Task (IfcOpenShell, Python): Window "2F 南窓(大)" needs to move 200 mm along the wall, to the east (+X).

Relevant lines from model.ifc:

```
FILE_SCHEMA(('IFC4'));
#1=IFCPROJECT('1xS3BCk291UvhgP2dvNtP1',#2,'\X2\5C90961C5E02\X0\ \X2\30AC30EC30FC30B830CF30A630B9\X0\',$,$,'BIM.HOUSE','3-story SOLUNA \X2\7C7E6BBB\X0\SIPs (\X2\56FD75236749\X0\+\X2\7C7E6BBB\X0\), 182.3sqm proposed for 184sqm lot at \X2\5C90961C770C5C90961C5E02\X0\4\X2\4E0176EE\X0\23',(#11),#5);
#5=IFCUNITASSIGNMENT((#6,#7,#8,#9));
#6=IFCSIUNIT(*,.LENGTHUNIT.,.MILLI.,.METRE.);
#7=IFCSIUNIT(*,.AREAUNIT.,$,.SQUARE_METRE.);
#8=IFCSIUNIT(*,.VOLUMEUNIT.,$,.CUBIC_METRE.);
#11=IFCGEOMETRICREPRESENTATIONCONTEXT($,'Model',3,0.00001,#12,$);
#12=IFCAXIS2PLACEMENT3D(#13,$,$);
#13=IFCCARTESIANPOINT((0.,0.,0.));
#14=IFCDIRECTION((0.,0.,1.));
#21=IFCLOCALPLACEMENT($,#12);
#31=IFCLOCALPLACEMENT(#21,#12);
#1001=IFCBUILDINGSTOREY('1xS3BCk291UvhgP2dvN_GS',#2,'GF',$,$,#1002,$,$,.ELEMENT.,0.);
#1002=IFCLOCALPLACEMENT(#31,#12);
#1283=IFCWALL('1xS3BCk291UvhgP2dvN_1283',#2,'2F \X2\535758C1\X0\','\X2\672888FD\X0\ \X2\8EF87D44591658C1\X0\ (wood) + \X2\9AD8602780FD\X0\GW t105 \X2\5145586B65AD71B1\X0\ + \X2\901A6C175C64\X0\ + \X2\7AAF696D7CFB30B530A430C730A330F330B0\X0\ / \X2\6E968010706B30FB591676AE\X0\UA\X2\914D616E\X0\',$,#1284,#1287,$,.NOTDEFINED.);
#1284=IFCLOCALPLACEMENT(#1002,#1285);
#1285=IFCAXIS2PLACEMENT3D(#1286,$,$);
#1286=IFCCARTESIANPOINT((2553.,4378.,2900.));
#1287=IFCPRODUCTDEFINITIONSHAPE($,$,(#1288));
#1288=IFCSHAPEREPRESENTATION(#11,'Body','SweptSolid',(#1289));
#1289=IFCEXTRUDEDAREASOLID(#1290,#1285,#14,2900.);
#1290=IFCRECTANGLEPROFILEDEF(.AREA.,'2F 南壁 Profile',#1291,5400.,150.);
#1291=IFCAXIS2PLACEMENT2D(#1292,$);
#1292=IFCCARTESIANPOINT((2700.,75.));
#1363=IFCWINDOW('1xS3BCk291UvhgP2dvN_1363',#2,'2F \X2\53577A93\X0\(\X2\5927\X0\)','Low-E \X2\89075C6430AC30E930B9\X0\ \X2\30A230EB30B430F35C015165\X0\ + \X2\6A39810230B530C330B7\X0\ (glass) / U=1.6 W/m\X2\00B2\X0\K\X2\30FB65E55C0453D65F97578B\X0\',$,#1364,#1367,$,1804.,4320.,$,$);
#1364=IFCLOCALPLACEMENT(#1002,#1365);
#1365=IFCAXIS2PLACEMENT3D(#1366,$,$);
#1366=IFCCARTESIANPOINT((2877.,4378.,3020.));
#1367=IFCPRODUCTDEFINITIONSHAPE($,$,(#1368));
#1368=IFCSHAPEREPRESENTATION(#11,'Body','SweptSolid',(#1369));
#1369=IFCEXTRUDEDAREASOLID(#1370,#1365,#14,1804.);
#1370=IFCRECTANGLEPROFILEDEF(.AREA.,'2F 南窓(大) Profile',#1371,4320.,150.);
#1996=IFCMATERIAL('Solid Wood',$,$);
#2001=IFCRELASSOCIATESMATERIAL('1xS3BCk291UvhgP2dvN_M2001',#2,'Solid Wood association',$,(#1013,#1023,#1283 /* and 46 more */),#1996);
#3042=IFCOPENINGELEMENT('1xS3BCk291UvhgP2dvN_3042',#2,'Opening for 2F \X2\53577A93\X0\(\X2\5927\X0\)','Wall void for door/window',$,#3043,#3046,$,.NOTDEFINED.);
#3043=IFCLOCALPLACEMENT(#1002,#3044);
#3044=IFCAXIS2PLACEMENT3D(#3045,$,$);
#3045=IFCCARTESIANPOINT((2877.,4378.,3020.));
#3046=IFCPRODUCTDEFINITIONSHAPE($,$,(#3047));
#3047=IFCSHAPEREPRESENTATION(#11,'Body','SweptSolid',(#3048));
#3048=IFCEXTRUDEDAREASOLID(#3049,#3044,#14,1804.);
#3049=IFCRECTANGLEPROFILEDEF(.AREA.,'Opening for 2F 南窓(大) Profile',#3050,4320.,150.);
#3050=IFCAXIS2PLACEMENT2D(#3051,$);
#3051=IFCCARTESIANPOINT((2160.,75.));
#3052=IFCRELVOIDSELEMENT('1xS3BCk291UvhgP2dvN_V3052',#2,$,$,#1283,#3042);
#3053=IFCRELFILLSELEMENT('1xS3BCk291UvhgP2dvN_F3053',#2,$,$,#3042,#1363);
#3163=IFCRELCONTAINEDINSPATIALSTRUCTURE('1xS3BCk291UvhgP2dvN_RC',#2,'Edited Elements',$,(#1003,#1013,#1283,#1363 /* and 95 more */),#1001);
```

```python
import ifcopenshell
import ifcopenshell.api.geometry
import ifcopenshell.util.placement
import ifcopenshell.util.unit

model = ifcopenshell.open("model.ifc")
unit_scale = ifcopenshell.util.unit.calculate_unit_scale(model)

window = model.by_guid("1xS3BCk291UvhgP2dvN_1363")
opening = window.FillsVoids[0].RelatingOpeningElement
wall = opening.VoidsElements[0].RelatingBuildingElement

wall_matrix = ifcopenshell.util.placement.get_local_placement(wall.ObjectPlacement)
shift = wall_matrix[:3, 0] * 0.2 / unit_scale
before = ifcopenshell.util.placement.get_local_placement(window.ObjectPlacement)[:3, 3].copy()

# The window is not placed relative to its opening, so move both.
for product in (opening, window):
    matrix = ifcopenshell.util.placement.get_local_placement(product.ObjectPlacement)
    matrix[:3, 3] += shift
    ifcopenshell.api.geometry.edit_object_placement(model, product=product, matrix=matrix, is_si=False)

after = ifcopenshell.util.placement.get_local_placement(window.ObjectPlacement)[:3, 3]
print("window moved by", (after - before).round(3) + 0.0)

model.write("model_updated.ifc")
```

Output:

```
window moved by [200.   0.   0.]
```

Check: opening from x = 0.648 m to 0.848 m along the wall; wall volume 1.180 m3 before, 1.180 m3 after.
